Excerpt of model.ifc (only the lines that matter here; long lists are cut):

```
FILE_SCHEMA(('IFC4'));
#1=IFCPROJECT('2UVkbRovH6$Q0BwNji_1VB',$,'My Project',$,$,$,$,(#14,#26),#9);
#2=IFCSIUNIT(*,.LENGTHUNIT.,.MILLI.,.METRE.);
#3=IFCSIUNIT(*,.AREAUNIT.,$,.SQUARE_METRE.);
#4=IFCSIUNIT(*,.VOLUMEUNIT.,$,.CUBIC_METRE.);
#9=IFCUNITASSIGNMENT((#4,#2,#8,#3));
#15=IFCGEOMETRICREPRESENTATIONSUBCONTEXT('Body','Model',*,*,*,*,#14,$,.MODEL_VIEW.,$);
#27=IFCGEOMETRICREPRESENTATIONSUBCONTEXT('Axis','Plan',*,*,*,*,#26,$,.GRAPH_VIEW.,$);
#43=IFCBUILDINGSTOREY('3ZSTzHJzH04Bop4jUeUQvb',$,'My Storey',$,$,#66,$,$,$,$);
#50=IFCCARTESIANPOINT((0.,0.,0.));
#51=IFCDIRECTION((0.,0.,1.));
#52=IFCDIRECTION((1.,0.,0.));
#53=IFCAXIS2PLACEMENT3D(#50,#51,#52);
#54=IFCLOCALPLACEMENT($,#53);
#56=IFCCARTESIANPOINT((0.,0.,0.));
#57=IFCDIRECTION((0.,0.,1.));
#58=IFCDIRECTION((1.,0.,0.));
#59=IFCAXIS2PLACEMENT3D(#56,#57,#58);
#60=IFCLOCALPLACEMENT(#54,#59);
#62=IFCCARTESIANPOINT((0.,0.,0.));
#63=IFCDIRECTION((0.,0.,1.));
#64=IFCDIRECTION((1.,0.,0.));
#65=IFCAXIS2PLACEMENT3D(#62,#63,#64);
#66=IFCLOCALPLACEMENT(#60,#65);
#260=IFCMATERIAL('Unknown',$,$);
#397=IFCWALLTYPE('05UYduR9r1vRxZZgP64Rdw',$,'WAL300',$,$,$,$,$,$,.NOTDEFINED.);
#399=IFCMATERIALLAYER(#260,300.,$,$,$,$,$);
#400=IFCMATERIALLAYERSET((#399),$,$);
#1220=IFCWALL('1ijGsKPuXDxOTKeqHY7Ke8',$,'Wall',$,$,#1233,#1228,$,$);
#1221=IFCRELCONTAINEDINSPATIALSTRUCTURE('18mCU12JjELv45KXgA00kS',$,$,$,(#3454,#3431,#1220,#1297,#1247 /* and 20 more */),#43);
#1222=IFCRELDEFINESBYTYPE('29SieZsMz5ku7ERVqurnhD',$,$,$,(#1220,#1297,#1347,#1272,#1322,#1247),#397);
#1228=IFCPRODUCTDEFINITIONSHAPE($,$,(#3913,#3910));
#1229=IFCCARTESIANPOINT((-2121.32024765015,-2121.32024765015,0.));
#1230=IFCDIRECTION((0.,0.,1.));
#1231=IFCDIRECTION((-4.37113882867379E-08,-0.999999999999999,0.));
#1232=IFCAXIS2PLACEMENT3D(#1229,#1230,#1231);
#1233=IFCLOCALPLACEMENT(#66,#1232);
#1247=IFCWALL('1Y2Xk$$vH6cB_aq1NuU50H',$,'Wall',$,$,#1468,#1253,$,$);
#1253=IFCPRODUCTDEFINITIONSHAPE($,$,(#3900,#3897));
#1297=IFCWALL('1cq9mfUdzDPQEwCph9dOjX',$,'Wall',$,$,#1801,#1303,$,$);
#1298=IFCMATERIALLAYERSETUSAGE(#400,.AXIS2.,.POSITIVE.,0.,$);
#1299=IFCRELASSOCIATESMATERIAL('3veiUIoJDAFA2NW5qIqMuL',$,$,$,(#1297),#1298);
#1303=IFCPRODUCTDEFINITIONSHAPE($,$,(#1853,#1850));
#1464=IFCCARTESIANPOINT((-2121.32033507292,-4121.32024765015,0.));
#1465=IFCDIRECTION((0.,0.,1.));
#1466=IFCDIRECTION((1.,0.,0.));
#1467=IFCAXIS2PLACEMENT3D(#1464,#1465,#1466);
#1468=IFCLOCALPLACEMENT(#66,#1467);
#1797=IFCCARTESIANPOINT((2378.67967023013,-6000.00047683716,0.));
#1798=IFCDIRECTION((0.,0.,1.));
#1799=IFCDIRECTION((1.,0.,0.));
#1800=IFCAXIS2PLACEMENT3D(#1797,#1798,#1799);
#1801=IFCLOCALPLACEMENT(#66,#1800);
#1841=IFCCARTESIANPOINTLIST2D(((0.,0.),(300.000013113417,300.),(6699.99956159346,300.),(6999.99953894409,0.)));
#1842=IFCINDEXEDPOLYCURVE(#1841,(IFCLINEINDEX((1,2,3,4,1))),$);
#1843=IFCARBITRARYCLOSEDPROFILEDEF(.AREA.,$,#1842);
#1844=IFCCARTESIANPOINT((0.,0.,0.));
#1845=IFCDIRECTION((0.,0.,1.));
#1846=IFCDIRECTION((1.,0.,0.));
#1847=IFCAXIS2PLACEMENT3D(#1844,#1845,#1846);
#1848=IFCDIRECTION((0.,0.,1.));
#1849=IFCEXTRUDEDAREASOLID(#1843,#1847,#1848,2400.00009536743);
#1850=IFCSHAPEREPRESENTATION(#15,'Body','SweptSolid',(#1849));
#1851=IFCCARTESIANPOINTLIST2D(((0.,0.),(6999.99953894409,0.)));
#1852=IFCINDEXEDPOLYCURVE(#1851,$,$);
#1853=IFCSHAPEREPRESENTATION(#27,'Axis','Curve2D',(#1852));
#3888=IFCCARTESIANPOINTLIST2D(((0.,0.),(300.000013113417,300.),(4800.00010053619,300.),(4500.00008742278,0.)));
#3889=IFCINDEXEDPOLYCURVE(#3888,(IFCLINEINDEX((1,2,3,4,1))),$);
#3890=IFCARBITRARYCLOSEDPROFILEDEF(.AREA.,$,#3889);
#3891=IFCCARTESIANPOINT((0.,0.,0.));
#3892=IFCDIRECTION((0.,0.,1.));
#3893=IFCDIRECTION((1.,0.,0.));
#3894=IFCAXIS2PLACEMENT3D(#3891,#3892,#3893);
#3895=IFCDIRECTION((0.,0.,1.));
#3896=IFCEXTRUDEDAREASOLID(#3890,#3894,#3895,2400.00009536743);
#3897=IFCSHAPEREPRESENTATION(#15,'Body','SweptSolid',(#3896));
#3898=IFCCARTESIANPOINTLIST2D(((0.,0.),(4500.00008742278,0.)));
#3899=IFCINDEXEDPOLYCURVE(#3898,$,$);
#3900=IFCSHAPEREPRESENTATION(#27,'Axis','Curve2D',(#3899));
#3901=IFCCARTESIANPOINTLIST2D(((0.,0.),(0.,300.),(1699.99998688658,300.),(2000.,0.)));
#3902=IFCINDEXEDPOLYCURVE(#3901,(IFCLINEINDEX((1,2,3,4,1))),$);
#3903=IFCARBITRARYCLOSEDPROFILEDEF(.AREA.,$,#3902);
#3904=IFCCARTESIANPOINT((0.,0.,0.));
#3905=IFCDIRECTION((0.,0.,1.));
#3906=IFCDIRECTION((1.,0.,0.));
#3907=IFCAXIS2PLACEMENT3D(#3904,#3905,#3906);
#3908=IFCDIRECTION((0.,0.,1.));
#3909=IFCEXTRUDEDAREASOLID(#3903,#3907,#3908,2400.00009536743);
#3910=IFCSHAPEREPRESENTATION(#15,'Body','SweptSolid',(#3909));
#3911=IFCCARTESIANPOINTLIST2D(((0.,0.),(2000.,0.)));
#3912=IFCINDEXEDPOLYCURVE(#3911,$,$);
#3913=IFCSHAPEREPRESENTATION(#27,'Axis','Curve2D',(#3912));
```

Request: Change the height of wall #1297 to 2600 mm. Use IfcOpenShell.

```python
import ifcopenshell
import ifcopenshell.geom
import ifcopenshell.util.representation
import ifcopenshell.util.shape

model = ifcopenshell.open("model.ifc")
settings = ifcopenshell.geom.settings()


def volume(element):
    """Net volume in cubic metres, openings subtracted."""
    shape = ifcopenshell.geom.create_shape(settings, element)
    return ifcopenshell.util.shape.get_volume(shape.geometry)


wall = model.by_guid("1cq9mfUdzDPQEwCph9dOjX")
before = volume(wall)

body = ifcopenshell.util.representation.get_representation(wall, "Model", "Body")
solid = body.Items[0]
old_height = solid.Depth
solid.Depth = 2600.0
after = volume(wall)

print(f"height {old_height:g} -> {solid.Depth:g}, volume {before:.3f} -> {after:.3f} m3")

model.write("model_rev.ifc")
```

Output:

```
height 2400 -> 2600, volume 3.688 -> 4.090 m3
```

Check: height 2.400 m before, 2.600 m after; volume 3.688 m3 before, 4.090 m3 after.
